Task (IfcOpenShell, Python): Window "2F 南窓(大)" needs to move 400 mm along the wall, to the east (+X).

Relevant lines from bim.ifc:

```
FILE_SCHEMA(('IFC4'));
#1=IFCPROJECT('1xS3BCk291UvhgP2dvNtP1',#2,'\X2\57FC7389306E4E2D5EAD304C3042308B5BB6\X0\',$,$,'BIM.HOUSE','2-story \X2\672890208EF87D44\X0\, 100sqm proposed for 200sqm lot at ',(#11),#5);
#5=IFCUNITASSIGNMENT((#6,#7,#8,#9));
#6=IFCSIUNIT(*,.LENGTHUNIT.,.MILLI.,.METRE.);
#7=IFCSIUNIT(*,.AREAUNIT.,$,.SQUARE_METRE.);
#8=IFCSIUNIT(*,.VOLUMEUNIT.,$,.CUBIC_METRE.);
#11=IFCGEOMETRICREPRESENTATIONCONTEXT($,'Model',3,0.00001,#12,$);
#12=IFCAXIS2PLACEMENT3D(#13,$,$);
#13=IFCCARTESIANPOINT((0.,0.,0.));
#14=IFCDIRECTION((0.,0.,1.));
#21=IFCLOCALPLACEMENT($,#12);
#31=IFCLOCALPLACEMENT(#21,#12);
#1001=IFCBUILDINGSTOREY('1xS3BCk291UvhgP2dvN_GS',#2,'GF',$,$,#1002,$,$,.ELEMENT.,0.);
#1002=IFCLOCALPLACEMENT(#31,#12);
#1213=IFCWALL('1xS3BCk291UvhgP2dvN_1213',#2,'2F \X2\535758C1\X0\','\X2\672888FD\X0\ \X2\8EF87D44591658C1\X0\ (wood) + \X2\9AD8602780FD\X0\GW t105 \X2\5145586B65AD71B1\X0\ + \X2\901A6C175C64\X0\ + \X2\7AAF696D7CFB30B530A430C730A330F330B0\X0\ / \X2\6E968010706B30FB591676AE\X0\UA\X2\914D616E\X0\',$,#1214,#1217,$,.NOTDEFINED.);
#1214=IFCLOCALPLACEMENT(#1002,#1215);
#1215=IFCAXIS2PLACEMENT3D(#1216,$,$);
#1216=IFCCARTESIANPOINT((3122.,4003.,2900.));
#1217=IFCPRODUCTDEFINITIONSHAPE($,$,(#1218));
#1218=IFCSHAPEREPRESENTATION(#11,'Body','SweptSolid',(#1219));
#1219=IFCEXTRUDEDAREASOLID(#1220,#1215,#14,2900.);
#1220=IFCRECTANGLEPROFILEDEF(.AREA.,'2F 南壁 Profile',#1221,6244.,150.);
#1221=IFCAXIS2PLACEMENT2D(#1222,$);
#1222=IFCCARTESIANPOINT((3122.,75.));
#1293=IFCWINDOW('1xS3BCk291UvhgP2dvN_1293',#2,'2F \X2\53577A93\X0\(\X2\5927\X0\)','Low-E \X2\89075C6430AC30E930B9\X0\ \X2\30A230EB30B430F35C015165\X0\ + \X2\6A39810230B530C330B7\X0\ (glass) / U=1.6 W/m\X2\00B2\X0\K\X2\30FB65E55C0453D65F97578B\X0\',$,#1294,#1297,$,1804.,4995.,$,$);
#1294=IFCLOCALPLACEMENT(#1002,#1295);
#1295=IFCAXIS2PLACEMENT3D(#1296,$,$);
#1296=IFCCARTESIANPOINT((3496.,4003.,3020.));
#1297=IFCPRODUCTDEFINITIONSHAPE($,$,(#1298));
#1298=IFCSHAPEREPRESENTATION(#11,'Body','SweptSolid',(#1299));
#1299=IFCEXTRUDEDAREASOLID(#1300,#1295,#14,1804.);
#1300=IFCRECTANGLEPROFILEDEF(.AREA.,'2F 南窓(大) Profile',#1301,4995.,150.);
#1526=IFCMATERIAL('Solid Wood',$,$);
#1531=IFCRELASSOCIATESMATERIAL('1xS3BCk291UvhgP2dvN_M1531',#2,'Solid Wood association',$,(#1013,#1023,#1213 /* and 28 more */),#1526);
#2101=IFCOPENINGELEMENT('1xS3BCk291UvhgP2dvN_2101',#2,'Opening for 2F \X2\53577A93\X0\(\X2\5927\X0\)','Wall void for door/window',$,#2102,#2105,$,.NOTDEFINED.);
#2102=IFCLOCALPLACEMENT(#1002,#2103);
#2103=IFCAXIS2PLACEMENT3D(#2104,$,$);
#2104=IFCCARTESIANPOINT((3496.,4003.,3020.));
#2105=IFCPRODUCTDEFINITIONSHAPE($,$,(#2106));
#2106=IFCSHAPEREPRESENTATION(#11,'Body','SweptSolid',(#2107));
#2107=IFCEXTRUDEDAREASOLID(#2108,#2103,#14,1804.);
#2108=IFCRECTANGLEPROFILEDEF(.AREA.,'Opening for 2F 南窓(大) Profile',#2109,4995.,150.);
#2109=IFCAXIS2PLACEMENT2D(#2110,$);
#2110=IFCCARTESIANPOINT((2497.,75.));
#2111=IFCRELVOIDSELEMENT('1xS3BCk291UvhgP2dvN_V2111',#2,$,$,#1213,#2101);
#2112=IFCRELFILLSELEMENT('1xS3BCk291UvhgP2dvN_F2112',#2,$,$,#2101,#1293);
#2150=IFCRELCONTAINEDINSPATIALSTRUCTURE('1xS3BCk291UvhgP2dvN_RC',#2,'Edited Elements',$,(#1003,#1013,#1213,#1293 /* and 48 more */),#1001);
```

```python
import ifcopenshell
import ifcopenshell.api.geometry
import ifcopenshell.util.placement
import ifcopenshell.util.unit

model = ifcopenshell.open("bim.ifc")
unit_scale = ifcopenshell.util.unit.calculate_unit_scale(model)

window = model.by_guid("1xS3BCk291UvhgP2dvN_1293")
opening = window.FillsVoids[0].RelatingOpeningElement
wall = opening.VoidsElements[0].RelatingBuildingElement

wall_matrix = ifcopenshell.util.placement.get_local_placement(wall.ObjectPlacement)
shift = wall_matrix[:3, 0] * 0.4 / unit_scale
before = ifcopenshell.util.placement.get_local_placement(window.ObjectPlacement)[:3, 3].copy()

# The window is not placed relative to its opening, so move both.
for product in (opening, window):
    matrix = ifcopenshell.util.placement.get_local_placement(product.ObjectPlacement)
    matrix[:3, 3] += shift
    ifcopenshell.api.geometry.edit_object_placement(model, product=product, matrix=matrix, is_si=False)

after = ifcopenshell.util.placement.get_local_placement(window.ObjectPlacement)[:3, 3]
print("window moved by", (after - before).round(3) + 0.0)

model.write("bim_edited.ifc")
```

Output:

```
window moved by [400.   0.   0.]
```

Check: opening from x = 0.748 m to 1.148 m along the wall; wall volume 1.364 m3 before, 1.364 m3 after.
